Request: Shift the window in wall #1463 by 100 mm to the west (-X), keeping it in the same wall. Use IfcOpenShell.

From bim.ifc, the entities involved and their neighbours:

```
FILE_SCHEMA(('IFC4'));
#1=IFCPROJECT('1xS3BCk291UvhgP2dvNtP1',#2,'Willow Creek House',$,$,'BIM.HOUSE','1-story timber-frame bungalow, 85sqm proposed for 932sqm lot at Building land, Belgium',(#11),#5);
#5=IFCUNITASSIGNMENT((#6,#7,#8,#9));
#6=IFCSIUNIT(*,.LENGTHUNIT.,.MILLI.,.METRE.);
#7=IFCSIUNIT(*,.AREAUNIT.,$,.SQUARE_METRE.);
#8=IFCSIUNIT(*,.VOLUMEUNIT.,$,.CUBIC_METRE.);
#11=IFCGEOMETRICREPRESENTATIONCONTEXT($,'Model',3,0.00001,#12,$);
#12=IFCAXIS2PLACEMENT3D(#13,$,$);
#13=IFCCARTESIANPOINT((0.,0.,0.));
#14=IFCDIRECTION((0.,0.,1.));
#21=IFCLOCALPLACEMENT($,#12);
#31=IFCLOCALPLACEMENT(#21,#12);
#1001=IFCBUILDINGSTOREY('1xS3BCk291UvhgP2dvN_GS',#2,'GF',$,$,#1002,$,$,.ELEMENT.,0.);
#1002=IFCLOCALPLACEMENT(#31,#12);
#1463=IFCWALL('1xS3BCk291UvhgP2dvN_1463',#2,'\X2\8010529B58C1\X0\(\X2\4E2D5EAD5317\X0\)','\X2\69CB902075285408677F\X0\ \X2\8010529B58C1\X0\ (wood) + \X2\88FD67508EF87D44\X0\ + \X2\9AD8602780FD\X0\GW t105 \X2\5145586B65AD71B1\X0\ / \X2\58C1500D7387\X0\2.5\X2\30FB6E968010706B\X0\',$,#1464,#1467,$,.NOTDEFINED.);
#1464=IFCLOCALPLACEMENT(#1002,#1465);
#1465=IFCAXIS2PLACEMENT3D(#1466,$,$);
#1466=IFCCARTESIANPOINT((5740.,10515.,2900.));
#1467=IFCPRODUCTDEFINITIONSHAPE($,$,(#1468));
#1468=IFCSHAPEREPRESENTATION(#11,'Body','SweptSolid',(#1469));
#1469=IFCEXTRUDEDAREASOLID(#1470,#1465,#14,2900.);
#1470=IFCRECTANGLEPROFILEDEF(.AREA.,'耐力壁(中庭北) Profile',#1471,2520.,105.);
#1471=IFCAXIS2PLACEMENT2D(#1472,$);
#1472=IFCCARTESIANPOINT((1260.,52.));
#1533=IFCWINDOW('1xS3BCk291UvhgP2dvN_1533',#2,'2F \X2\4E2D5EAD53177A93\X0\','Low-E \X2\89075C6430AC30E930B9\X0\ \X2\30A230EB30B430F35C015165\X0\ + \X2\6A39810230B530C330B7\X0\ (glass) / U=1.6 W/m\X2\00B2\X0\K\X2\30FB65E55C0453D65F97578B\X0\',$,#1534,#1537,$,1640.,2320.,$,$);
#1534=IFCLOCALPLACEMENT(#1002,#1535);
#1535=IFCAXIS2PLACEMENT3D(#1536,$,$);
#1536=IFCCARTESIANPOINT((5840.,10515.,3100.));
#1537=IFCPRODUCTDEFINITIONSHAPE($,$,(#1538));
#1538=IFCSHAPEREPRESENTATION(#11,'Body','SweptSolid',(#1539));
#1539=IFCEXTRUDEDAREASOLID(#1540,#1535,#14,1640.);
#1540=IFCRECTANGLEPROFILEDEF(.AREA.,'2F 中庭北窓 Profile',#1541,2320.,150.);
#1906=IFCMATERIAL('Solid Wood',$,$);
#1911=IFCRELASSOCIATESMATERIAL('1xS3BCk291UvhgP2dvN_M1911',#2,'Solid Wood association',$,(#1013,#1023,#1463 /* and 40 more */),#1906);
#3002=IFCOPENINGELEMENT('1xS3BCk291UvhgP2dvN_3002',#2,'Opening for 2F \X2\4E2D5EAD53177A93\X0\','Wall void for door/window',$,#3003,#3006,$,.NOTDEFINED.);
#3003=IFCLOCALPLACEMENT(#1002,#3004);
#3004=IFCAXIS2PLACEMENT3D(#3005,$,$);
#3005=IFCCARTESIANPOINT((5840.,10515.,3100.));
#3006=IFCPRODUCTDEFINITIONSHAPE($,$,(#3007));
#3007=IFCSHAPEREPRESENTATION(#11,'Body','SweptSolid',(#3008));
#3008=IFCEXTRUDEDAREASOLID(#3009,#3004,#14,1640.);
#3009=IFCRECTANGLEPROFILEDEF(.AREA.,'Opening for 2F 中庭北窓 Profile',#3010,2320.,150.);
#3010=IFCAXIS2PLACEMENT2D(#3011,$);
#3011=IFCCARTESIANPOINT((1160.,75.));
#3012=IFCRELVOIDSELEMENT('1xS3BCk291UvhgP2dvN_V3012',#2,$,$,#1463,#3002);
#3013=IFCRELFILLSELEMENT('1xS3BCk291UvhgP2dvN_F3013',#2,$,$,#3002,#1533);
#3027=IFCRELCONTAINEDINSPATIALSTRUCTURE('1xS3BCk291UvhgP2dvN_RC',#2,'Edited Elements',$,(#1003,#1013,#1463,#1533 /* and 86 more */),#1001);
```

```python
import ifcopenshell
import ifcopenshell.api.geometry
import ifcopenshell.util.placement

model = ifcopenshell.open("bim.ifc")

window = model.by_guid("1xS3BCk291UvhgP2dvN_1533")
opening = window.FillsVoids[0].RelatingOpeningElement
wall = opening.VoidsElements[0].RelatingBuildingElement

wall_matrix = ifcopenshell.util.placement.get_local_placement(wall.ObjectPlacement)
shift = wall_matrix[:3, 0] * -100.0
before = ifcopenshell.util.placement.get_local_placement(window.ObjectPlacement)[:3, 3].copy()

# The window is not placed relative to its opening, so move both.
for product in (opening, window):
    matrix = ifcopenshell.util.placement.get_local_placement(product.ObjectPlacement)
    matrix[:3, 3] += shift
    ifcopenshell.api.geometry.edit_object_placement(model, product=product, matrix=matrix, is_si=False)

after = ifcopenshell.util.placement.get_local_placement(window.ObjectPlacement)[:3, 3]
print("window moved by", (after - before).round(3) + 0.0)

model.write("bim_updated.ifc")
```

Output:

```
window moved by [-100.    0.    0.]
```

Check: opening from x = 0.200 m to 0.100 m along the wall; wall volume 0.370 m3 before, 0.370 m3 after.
